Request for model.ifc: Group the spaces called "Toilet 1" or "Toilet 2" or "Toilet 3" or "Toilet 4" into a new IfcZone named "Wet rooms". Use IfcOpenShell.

First a look at what the model holds.

```python
import ifcopenshell

model = ifcopenshell.open("model.ifc")
print(model.schema)
seen = {}
for space in model.by_type("IfcSpace"):
    seen[space.LongName] = seen.get(space.LongName, 0) + 1
for name, count in sorted(seen.items(), key=str):
    print(count, "x", name)
print("zones:", [z.Name for z in model.by_type("IfcZone")][:20])
```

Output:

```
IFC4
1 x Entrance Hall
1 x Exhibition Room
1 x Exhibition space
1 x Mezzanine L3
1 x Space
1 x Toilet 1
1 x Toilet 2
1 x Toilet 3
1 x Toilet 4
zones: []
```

```python
import ifcopenshell
import ifcopenshell.api.group
import ifcopenshell.api.root

model = ifcopenshell.open("model.ifc")

names = {"Toilet 1", "Toilet 2", "Toilet 3", "Toilet 4"}
spaces = [s for s in model.by_type("IfcSpace") if s.LongName in names]

zone = ifcopenshell.api.root.create_entity(model, ifc_class="IfcZone", name="Wet rooms")
ifcopenshell.api.group.assign_group(model, products=spaces, group=zone)
print(len(spaces), "spaces in", zone.Name)

model.write("model_edited.ifc")
```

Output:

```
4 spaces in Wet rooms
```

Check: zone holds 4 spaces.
